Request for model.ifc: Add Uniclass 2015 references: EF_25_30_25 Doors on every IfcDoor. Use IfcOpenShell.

First a look at what the model holds.

```python
import ifcopenshell

model = ifcopenshell.open("model.ifc")
print(model.schema)
print("classifications:", [c.Name for c in model.by_type("IfcClassification")])
for ifc_class in ("IfcDoor", "IfcRoof", "IfcStair", "IfcWall", "IfcWindow"):
    print(ifc_class, len(model.by_type(ifc_class)))
```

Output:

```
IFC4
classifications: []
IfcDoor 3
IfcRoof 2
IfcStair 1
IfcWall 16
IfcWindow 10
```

```python
import ifcopenshell
import ifcopenshell.api.classification

model = ifcopenshell.open("model.ifc")

system = ifcopenshell.api.classification.add_classification(model, classification="Uniclass 2015")

codes = {
    "IfcDoor": ("EF_25_30_25", "Doors"),
}
for ifc_class, (code, name) in codes.items():
    products = model.by_type(ifc_class)
    ifcopenshell.api.classification.add_reference(
        model, products=products, classification=system, identification=code, name=name
    )
    print(code, len(products))

model.write("model_edited.ifc")
```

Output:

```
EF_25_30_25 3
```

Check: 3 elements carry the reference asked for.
